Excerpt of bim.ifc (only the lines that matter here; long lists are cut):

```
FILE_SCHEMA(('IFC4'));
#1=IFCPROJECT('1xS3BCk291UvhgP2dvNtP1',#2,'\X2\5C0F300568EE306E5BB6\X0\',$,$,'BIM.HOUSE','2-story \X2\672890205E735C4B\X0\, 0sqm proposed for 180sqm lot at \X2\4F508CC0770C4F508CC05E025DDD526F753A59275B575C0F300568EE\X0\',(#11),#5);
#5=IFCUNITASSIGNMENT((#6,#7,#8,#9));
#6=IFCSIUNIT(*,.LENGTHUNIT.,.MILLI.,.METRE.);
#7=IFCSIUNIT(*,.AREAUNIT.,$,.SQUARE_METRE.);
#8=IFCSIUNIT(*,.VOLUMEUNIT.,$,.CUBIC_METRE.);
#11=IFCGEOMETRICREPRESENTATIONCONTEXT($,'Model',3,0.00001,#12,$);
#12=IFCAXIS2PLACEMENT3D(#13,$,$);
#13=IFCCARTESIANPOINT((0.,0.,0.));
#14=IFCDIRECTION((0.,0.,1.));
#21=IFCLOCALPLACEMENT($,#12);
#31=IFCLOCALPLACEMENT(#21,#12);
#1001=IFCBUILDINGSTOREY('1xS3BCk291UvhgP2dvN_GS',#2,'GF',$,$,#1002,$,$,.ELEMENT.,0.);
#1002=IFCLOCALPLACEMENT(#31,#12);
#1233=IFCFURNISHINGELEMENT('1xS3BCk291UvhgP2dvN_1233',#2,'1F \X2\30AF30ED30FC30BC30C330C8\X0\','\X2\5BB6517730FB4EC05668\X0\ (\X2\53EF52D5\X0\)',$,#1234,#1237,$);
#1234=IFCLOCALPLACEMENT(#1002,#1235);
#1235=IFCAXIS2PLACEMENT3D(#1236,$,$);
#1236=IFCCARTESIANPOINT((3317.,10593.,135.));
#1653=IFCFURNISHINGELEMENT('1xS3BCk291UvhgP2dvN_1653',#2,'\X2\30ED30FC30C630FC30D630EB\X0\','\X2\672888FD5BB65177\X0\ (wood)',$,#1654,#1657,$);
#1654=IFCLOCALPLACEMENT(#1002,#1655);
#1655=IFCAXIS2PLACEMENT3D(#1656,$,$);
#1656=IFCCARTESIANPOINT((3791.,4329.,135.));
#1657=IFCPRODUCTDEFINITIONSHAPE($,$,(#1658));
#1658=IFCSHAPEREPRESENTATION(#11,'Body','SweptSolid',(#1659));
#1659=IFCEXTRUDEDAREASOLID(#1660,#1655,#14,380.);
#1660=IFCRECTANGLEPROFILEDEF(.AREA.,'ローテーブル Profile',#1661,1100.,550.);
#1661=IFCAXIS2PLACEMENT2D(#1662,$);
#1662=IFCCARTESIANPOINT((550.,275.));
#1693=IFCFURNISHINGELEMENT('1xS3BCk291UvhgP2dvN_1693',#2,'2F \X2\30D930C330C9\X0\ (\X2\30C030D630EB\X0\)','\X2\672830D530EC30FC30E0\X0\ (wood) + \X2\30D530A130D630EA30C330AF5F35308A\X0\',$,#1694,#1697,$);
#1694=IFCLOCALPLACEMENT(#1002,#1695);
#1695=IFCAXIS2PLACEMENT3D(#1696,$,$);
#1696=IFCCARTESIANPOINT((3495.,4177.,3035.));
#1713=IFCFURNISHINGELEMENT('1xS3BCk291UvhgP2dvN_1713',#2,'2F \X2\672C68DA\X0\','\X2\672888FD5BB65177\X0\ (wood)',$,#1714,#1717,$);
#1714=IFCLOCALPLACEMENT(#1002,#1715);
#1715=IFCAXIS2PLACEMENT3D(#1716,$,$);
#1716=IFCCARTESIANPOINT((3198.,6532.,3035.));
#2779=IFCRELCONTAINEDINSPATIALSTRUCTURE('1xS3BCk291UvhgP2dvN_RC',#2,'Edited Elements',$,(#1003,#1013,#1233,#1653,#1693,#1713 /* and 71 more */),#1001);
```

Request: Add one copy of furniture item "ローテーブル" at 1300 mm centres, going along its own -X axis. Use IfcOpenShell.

```python
import ifcopenshell
import ifcopenshell.api.geometry
import ifcopenshell.api.root
import ifcopenshell.util.element
import ifcopenshell.util.placement
import ifcopenshell.util.unit

model = ifcopenshell.open("bim.ifc")
unit_scale = ifcopenshell.util.unit.calculate_unit_scale(model)


def reuse_history(source, copy):
    """copy_class also copies each property set's owner history, people and application; keep the originals."""
    for rel in copy.IsDefinedBy:
        if rel.is_a("IfcRelDefinesByProperties") and (history := rel.RelatingPropertyDefinition.OwnerHistory):
            rel.RelatingPropertyDefinition.OwnerHistory = source.OwnerHistory
            ifcopenshell.util.element.remove_deep2(model, history)


source = model.by_guid("1xS3BCk291UvhgP2dvN_1653")
base = ifcopenshell.util.placement.get_local_placement(source.ObjectPlacement)
step = -base[:3, 0] * 1.3 / unit_scale

for i in range(1, 2):
    copy = ifcopenshell.api.root.copy_class(model, product=source)
    copy.Representation = ifcopenshell.util.element.copy_deep(
        model, source.Representation, exclude=["IfcGeometricRepresentationContext", "IfcRepresentationMap"]
    )
    reuse_history(source, copy)
    matrix = base.copy()
    matrix[:3, 3] += i * step
    print("added at", matrix[:3, 3].round(3) + 0.0)
    ifcopenshell.api.geometry.edit_object_placement(model, product=copy, matrix=matrix, is_si=False)

model.write("bim-out.ifc")
```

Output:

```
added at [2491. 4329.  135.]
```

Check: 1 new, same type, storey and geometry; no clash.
